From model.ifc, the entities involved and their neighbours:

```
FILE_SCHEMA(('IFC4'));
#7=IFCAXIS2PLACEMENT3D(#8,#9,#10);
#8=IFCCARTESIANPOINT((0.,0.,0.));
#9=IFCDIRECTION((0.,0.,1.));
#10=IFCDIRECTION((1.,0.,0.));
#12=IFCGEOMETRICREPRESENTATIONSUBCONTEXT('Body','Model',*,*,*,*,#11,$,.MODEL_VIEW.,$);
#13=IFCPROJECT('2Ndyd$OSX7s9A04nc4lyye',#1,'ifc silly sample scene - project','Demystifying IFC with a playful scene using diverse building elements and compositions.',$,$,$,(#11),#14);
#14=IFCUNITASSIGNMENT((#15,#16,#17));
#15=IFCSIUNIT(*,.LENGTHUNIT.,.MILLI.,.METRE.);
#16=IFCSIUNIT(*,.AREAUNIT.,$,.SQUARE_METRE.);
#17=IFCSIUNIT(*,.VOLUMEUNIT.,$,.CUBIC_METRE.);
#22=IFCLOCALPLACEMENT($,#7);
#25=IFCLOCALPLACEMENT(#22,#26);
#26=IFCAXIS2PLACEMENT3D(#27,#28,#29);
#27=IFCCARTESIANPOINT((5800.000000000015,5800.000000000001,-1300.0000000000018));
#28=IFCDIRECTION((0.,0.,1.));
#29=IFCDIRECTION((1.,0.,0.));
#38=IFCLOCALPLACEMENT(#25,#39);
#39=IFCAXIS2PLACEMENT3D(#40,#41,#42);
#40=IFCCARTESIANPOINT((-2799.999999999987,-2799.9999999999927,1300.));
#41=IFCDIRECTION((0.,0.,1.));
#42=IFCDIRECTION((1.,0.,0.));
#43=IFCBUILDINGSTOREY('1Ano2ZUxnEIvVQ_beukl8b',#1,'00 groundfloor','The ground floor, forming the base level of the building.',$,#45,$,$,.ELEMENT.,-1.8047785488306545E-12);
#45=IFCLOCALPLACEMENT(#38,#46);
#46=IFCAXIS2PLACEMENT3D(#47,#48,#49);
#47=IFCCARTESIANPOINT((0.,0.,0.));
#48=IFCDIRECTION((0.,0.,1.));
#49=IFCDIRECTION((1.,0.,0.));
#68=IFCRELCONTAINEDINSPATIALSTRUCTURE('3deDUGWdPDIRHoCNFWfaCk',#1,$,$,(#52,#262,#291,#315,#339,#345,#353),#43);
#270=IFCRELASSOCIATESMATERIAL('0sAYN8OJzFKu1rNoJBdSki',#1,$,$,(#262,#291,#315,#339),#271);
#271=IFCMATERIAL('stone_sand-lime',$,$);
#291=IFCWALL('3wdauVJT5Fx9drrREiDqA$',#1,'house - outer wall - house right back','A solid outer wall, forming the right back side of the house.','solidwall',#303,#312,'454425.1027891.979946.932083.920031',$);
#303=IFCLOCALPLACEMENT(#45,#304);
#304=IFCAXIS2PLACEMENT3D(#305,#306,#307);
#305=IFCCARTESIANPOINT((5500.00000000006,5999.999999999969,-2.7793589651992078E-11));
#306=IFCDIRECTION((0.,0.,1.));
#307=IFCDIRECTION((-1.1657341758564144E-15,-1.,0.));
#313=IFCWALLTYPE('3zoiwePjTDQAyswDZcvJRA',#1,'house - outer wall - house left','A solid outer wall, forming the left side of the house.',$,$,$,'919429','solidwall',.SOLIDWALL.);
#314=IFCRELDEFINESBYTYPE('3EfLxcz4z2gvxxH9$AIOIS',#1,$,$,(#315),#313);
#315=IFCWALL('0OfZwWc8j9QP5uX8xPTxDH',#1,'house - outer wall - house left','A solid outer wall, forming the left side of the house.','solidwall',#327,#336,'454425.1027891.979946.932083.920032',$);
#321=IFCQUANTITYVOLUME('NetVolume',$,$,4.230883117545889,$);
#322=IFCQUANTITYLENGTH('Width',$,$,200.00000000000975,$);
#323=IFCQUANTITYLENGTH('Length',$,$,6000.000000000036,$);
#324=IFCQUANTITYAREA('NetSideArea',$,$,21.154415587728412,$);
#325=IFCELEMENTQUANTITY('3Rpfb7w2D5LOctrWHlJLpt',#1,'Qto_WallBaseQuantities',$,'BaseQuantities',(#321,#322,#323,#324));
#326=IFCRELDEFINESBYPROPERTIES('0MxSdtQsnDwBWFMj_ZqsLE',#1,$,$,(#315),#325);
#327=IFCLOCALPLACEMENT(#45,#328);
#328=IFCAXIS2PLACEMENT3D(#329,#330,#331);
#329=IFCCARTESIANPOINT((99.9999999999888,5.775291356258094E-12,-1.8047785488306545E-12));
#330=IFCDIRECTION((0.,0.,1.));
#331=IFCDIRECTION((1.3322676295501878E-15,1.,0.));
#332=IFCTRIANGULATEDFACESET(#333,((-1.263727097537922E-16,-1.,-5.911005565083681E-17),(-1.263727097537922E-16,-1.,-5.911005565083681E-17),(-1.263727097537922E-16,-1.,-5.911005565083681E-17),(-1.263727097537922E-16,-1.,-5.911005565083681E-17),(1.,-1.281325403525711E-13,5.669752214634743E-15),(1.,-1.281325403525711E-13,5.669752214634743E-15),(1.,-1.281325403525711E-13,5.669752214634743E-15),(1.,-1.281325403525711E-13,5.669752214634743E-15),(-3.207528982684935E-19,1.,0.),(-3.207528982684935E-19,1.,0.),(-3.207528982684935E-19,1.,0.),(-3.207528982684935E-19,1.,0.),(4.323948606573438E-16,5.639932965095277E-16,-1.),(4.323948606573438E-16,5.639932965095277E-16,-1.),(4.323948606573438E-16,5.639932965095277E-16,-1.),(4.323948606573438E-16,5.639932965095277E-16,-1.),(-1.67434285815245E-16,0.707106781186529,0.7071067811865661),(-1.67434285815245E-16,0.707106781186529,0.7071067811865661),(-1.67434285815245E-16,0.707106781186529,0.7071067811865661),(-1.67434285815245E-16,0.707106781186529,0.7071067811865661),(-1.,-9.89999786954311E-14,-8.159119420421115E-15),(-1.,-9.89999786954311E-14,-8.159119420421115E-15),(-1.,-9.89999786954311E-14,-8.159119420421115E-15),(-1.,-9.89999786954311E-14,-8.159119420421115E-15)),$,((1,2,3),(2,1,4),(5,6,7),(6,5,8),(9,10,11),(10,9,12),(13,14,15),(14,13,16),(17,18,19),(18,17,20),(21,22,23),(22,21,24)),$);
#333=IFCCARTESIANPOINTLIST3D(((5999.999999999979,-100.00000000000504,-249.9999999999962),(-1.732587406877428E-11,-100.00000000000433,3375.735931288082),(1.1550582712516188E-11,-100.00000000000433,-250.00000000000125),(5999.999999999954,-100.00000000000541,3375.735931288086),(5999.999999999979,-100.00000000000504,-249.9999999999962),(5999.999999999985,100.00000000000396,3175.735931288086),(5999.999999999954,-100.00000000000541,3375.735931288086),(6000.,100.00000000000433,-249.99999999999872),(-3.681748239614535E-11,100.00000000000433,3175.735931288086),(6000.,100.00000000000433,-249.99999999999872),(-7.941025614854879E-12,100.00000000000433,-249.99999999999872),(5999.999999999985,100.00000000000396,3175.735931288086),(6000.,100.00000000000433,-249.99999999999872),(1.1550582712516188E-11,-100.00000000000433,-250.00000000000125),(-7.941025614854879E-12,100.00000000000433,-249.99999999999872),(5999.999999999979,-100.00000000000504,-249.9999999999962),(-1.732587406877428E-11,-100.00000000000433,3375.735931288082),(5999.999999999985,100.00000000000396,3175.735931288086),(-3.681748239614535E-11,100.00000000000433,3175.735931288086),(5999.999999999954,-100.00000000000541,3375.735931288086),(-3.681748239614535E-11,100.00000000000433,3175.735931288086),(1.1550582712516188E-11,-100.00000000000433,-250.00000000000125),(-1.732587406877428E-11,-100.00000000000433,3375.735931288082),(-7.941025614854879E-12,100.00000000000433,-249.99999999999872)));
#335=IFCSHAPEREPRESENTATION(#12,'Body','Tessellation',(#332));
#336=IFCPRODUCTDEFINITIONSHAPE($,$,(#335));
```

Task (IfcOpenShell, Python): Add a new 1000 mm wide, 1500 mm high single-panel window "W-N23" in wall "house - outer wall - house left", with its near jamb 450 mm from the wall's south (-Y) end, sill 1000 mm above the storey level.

```python
import numpy as np
import ifcopenshell
import ifcopenshell.api.feature
import ifcopenshell.api.geometry
import ifcopenshell.api.pset
import ifcopenshell.api.root
import ifcopenshell.api.spatial
import ifcopenshell.geom
import ifcopenshell.util.element
import ifcopenshell.util.placement
import ifcopenshell.util.representation
import ifcopenshell.util.shape
import ifcopenshell.util.unit

model = ifcopenshell.open("model.ifc")
unit_scale = ifcopenshell.util.unit.calculate_unit_scale(model)
area_scale = ifcopenshell.util.unit.calculate_unit_scale(model, "AREAUNIT")
volume_scale = ifcopenshell.util.unit.calculate_unit_scale(model, "VOLUMEUNIT")
settings = ifcopenshell.geom.settings()


def volume(element):
    """Net volume in cubic metres, openings subtracted."""
    shape = ifcopenshell.geom.create_shape(settings, element)
    return ifcopenshell.util.shape.get_volume(shape.geometry)


wall = model.by_guid("0OfZwWc8j9QP5uX8xPTxDH")
storey = ifcopenshell.util.element.get_container(wall, ifc_class="IfcBuildingStorey")
context = ifcopenshell.util.representation.get_context(model, "Model", "Body", "MODEL_VIEW")
before = volume(wall)

width, height, from_end, sill = 1, 1.5, 0.45, 1  # metres

# The wall runs along its own X axis, and the end named is its -X end.
wall_shape = ifcopenshell.geom.create_shape(settings, wall)
x, y, z = ifcopenshell.util.shape.get_vertices(wall_shape.geometry).T
start = x.min() + from_end
face, thickness = float(y.min()), float(y.max() - y.min())
wall_matrix = ifcopenshell.util.placement.get_local_placement(wall.ObjectPlacement)
level = ifcopenshell.util.placement.get_local_placement(storey.ObjectPlacement)[2, 3]


def in_wall(x, y):
    """Placement at x, y metres in the wall's axes, at sill height."""
    matrix = wall_matrix.copy()
    matrix[:, 3] = wall_matrix @ np.array([x / unit_scale, y / unit_scale, 0.0, 1.0])
    matrix[2, 3] = level + sill / unit_scale
    return matrix


# Opening: a box that overshoots both wall faces by 50 mm.
opening = ifcopenshell.api.root.create_entity(model, ifc_class="IfcOpeningElement", predefined_type="OPENING")
box = ifcopenshell.api.geometry.add_wall_representation(
    model, context=context, length=width, height=height, thickness=thickness + 0.1
)
ifcopenshell.api.geometry.assign_representation(model, product=opening, representation=box)
ifcopenshell.api.geometry.edit_object_placement(model, product=opening, matrix=in_wall(start, face - 0.05), is_si=False)
ifcopenshell.api.feature.add_feature(model, feature=opening, element=wall)

window = ifcopenshell.api.root.create_entity(model, ifc_class="IfcWindow", name="W-N23", predefined_type="WINDOW")
window.OverallWidth, window.OverallHeight = width / unit_scale, height / unit_scale
window.PartitioningType = "SINGLE_PANEL"
body = ifcopenshell.api.geometry.add_window_representation(
    model,
    context=context,
    overall_width=window.OverallWidth,
    overall_height=window.OverallHeight,
    partition_type="SINGLE_PANEL",
)
ifcopenshell.api.geometry.assign_representation(model, product=window, representation=body)
ifcopenshell.api.spatial.assign_container(model, products=[window], relating_structure=storey)
ifcopenshell.api.feature.add_filling(model, opening=opening, element=window)

# Centre the window in the wall's thickness.
ifcopenshell.api.geometry.edit_object_placement(model, product=window, matrix=in_wall(start, face), is_si=False)
window_shape = ifcopenshell.geom.create_shape(settings, window)
depth = ifcopenshell.util.shape.get_vertices(window_shape.geometry)[:, 1]
offset = face + thickness / 2 - (depth.min() + depth.max()) / 2
ifcopenshell.api.geometry.edit_object_placement(model, product=window, matrix=in_wall(start, offset), is_si=False)

after = volume(wall)

# Update the wall's stored quantities.
qto = model.by_id(ifcopenshell.util.element.get_pset(wall, "Qto_WallBaseQuantities", should_inherit=False)["id"])
ifcopenshell.api.pset.edit_qto(model, qto=qto, properties={
    "NetVolume": after / volume_scale,
    "NetSideArea": after / thickness / area_scale,
})

print(f"wall volume {before:.3f} -> {after:.3f} m3")

model.write("model-out.ifc")
```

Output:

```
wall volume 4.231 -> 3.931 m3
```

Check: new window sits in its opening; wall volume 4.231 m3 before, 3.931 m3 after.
